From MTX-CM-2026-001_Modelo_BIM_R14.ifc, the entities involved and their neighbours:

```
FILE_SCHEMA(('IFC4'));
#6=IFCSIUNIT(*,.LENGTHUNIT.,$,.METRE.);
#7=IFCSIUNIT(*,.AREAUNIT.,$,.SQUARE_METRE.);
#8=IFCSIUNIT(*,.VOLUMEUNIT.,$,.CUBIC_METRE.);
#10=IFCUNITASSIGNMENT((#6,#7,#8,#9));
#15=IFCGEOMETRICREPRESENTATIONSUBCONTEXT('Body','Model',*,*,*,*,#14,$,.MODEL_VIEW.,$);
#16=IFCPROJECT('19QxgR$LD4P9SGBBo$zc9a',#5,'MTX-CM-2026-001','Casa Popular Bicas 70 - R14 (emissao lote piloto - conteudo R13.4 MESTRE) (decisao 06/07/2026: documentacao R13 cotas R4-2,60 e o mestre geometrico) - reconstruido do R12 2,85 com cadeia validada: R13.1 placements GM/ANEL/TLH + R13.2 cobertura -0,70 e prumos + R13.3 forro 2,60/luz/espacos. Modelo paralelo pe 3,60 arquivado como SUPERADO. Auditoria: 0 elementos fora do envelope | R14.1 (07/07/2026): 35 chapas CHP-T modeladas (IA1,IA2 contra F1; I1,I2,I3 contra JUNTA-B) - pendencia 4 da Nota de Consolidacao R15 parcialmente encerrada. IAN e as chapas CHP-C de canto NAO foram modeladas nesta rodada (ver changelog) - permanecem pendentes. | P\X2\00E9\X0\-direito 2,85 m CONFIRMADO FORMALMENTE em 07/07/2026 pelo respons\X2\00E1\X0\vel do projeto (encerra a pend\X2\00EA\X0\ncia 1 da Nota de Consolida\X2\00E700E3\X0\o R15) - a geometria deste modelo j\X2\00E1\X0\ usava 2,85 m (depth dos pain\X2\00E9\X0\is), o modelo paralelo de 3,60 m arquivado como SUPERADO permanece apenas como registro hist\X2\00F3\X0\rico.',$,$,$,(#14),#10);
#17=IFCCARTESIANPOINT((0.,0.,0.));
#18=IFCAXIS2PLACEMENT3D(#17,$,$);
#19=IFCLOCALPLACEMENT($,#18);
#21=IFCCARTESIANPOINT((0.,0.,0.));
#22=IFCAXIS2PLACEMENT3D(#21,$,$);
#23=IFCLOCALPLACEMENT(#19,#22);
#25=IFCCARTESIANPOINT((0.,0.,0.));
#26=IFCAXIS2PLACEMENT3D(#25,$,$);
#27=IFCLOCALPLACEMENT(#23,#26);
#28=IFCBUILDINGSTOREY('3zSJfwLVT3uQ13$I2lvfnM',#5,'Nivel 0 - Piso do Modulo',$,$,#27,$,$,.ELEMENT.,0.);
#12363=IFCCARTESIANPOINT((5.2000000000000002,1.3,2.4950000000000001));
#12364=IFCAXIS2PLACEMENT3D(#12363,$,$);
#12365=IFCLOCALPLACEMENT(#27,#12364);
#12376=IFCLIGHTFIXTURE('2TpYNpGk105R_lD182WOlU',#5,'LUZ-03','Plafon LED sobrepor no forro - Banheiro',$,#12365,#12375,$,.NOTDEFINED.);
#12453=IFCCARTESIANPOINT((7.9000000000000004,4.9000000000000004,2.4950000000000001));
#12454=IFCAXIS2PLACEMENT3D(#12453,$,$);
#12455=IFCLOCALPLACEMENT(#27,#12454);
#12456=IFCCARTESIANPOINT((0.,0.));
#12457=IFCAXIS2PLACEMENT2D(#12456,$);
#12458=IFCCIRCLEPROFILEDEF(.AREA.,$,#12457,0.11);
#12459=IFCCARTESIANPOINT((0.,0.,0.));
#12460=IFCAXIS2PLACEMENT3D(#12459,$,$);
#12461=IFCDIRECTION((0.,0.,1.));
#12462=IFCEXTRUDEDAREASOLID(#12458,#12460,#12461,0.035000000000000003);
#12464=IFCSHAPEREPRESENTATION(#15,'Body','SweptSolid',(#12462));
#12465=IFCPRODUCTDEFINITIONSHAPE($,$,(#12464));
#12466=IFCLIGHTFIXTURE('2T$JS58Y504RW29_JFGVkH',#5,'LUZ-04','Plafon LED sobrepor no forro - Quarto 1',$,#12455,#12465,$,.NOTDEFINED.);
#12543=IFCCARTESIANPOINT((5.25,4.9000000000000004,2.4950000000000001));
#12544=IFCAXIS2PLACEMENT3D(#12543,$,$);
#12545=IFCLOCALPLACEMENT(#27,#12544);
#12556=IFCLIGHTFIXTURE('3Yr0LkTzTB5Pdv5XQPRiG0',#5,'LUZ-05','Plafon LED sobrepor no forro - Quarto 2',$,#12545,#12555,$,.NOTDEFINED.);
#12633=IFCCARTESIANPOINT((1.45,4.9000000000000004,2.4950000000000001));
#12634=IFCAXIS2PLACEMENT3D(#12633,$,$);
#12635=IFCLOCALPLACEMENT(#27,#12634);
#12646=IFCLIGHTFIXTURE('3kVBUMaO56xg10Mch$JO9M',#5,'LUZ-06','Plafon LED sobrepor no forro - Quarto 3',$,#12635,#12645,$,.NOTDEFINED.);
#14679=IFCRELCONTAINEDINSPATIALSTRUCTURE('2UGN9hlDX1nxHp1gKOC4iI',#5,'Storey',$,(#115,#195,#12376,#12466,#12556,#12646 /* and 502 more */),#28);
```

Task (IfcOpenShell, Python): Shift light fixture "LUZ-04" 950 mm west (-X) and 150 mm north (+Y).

```python
import ifcopenshell
import ifcopenshell.api.geometry
import ifcopenshell.util.placement

model = ifcopenshell.open("MTX-CM-2026-001_Modelo_BIM_R14.ifc")

item = model.by_guid("2T$JS58Y504RW29_JFGVkH")
matrix = ifcopenshell.util.placement.get_local_placement(item.ObjectPlacement)
matrix[0, 3] -= 0.95
matrix[1, 3] += 0.15
ifcopenshell.api.geometry.edit_object_placement(model, product=item, matrix=matrix, is_si=False)

print(ifcopenshell.util.placement.get_local_placement(item.ObjectPlacement).round(3) + 0.0)

model.write("MTX-CM-2026-001_Modelo_BIM_R14_edited.ifc")
```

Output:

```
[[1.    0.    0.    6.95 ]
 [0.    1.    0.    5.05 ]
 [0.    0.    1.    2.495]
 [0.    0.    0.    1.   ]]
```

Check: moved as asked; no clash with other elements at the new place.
